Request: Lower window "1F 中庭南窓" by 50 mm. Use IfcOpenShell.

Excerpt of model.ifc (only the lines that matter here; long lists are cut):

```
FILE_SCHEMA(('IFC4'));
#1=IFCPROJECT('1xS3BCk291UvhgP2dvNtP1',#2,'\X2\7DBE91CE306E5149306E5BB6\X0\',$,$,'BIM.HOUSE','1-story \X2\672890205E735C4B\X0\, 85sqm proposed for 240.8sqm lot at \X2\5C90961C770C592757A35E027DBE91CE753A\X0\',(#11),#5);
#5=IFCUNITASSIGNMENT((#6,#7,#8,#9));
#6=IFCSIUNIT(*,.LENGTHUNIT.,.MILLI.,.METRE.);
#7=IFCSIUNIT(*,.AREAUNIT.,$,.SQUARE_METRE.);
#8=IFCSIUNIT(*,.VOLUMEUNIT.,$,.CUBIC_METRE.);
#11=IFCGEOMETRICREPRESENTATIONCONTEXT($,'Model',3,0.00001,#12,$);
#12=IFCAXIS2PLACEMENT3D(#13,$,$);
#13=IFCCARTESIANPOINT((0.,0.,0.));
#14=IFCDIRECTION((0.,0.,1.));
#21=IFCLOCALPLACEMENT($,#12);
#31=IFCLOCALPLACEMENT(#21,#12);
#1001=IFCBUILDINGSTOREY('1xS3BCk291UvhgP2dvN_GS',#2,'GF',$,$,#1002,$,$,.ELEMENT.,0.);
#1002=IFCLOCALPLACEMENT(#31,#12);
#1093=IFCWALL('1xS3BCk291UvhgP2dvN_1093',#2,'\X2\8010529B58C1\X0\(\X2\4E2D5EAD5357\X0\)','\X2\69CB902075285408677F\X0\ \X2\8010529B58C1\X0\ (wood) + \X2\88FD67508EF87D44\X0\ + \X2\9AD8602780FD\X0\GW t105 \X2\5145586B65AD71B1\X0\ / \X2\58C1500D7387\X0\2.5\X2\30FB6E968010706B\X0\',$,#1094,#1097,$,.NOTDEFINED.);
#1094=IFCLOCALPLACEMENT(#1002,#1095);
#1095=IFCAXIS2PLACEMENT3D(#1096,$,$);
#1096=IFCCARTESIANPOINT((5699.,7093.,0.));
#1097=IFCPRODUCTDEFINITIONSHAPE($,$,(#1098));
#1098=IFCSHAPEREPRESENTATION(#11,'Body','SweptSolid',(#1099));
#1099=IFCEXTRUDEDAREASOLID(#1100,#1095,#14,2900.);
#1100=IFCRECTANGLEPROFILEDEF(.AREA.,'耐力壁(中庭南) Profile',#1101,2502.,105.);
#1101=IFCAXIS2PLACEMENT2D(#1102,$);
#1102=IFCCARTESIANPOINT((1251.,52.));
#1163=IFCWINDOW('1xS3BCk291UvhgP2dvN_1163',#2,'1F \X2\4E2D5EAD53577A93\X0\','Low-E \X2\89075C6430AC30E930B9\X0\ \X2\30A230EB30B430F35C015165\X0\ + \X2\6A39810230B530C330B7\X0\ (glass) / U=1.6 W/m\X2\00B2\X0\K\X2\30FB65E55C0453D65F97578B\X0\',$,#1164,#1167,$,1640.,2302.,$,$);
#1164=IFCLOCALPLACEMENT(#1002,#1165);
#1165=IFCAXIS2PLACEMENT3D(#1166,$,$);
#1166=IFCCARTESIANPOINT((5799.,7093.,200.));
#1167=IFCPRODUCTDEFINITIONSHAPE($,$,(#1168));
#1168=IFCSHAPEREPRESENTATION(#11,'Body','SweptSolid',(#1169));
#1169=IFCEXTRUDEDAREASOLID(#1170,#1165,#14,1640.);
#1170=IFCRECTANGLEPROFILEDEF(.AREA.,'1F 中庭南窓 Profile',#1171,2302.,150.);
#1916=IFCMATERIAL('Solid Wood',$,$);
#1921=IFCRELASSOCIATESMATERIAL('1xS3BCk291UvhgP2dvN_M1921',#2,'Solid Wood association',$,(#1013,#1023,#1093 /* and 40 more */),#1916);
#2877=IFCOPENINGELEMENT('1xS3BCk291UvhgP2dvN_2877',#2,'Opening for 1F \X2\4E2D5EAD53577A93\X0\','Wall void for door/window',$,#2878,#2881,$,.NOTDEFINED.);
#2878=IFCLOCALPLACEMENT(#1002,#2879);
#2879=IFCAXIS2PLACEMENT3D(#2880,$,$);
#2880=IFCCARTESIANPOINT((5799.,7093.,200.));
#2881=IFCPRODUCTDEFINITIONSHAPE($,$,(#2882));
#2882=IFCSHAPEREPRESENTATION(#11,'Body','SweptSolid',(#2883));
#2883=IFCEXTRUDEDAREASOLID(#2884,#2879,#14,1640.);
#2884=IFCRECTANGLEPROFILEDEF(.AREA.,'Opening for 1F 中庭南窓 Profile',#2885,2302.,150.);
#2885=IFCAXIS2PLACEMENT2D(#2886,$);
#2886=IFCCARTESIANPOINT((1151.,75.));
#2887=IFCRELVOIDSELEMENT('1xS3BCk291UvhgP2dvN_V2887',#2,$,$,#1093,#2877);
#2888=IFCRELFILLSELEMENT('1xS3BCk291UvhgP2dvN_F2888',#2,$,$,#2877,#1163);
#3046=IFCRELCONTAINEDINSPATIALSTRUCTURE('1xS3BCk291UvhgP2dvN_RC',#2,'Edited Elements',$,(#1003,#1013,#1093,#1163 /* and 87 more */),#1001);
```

```python
import numpy as np
import ifcopenshell
import ifcopenshell.api.geometry
import ifcopenshell.util.placement
import ifcopenshell.util.unit

model = ifcopenshell.open("model.ifc")
unit_scale = ifcopenshell.util.unit.calculate_unit_scale(model)

window = model.by_guid("1xS3BCk291UvhgP2dvN_1163")
opening = window.FillsVoids[0].RelatingOpeningElement
dz = -0.05 / unit_scale

shift = np.array([0.0, 0.0, dz])
# The window is not placed relative to its opening, so move both.
for product in (opening, window):
    matrix = ifcopenshell.util.placement.get_local_placement(product.ObjectPlacement)
    matrix[:3, 3] += shift
    ifcopenshell.api.geometry.edit_object_placement(model, product=product, matrix=matrix, is_si=False)

print(f"moved by {dz * unit_scale:+.3f} m")

model.write("model_rev.ifc")
```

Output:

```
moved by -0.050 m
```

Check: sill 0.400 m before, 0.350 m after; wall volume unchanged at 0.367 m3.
